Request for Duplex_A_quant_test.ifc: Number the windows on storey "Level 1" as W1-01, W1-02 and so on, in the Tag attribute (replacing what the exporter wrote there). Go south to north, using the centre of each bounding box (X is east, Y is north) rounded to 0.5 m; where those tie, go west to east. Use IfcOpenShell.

First a look at what the model holds.

```python
import ifcopenshell
import ifcopenshell.util.element
import ifcopenshell.util.placement

model = ifcopenshell.open("Duplex_A_quant_test.ifc")
print(model.schema)
storey = next(s for s in model.by_type("IfcBuildingStorey") if s.Name == "Level 1")
windows = [e for e in ifcopenshell.util.element.get_decomposition(storey) if e.is_a("IfcWindow")]
for e in sorted(windows, key=lambda e: e.id()):
    origin = ifcopenshell.util.placement.get_local_placement(e.ObjectPlacement)[:3, 3]
    print(e.id(), e.Tag, e.Name, origin.round(2) + 0.0, sep=" | ")
```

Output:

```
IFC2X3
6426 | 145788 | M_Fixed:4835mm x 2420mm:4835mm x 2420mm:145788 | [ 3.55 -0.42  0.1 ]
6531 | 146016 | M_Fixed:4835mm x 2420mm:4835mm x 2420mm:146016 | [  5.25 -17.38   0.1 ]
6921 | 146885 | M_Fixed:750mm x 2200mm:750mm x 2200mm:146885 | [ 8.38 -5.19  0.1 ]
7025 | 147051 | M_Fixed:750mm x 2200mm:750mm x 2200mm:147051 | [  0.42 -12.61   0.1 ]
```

```python
import ifcopenshell
import ifcopenshell.geom
import ifcopenshell.util.element
import ifcopenshell.util.shape

model = ifcopenshell.open("Duplex_A_quant_test.ifc")
settings = ifcopenshell.geom.settings()
settings.set("use-world-coords", True)


def centre(element):
    shape = ifcopenshell.geom.create_shape(settings, element)
    return ifcopenshell.util.shape.get_bbox_centroid(shape.geometry)


storey = next(s for s in model.by_type("IfcBuildingStorey") if s.Name == "Level 1")
windows = [e for e in ifcopenshell.util.element.get_decomposition(storey) if e.is_a("IfcWindow")]

# Insertion points can sit at a corner or the storey origin, so sort by the geometry (in metres).
centres = {e: centre(e) for e in windows}
windows.sort(key=lambda e: (round(centres[e][1] / 0.5), centres[e][0]))

for i, e in enumerate(windows, start=1):
    number = f"W1-{i:02d}"
    e.Tag = number
    print(e.id(), number)

model.write("Duplex_A_quant_test_edited.ifc")
```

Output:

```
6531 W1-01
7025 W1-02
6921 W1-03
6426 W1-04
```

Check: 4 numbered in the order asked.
